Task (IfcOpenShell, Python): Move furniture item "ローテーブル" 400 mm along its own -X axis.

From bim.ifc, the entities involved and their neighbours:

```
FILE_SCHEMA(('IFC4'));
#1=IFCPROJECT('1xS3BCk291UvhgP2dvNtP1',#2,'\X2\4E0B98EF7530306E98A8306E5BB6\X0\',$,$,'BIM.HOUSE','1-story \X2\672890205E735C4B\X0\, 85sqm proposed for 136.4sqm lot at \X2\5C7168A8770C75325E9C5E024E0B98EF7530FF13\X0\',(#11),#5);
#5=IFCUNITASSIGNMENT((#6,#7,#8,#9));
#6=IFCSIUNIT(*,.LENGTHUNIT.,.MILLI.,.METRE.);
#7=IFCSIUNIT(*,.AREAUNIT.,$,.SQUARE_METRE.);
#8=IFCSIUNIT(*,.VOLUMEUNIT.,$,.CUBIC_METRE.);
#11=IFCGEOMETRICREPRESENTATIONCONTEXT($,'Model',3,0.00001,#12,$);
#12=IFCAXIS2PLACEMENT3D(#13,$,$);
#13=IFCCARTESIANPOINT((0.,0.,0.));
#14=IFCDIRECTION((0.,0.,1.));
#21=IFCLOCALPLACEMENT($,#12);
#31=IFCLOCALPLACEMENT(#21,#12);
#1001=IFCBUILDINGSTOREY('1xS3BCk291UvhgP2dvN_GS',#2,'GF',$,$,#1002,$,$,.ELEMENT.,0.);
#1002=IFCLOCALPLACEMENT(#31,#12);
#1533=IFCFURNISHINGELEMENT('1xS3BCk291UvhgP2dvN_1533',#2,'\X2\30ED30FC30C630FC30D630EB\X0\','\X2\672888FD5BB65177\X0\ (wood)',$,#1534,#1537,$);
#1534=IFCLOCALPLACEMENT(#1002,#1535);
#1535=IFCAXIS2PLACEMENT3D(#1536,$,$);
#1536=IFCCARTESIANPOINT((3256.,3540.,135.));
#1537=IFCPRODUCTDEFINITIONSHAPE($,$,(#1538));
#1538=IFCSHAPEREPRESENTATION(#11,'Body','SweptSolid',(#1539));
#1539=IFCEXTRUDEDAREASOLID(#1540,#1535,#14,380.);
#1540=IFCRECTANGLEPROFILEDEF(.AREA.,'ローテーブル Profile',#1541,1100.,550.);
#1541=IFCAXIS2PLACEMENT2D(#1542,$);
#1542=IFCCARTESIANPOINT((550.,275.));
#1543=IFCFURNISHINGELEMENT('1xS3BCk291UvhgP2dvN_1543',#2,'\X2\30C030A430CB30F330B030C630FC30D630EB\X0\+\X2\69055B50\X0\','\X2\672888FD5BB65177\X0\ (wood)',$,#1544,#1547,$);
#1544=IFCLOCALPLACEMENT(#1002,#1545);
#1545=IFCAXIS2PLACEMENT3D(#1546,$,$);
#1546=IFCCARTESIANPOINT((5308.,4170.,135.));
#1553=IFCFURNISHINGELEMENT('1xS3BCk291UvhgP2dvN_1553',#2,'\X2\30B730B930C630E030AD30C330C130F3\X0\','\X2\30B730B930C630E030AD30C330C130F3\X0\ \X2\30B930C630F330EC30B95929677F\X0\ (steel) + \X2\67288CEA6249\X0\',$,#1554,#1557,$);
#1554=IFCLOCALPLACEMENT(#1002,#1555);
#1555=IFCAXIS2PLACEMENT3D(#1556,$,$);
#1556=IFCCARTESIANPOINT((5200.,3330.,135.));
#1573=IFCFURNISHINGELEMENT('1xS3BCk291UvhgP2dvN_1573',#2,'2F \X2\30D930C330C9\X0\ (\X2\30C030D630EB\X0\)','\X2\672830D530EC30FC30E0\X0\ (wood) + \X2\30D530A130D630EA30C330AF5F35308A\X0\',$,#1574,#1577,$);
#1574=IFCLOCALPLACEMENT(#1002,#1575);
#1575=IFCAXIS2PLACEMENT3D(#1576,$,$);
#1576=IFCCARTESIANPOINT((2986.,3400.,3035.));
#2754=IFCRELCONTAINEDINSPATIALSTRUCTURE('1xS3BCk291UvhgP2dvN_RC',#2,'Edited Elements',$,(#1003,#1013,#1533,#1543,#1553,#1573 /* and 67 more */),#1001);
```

```python
import ifcopenshell
import ifcopenshell.api.geometry
import ifcopenshell.util.placement
import ifcopenshell.util.unit

model = ifcopenshell.open("bim.ifc")
unit_scale = ifcopenshell.util.unit.calculate_unit_scale(model)

item = model.by_guid("1xS3BCk291UvhgP2dvN_1533")
matrix = ifcopenshell.util.placement.get_local_placement(item.ObjectPlacement)
matrix[:3, 3] -= matrix[:3, 0] * 0.4 / unit_scale
ifcopenshell.api.geometry.edit_object_placement(model, product=item, matrix=matrix, is_si=False)

print(ifcopenshell.util.placement.get_local_placement(item.ObjectPlacement).round(3) + 0.0)

model.write("bim_rev.ifc")
```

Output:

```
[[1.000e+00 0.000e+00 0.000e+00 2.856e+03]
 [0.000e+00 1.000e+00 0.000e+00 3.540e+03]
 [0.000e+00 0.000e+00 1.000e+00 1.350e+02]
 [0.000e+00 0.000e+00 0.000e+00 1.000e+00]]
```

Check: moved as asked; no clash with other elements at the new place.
